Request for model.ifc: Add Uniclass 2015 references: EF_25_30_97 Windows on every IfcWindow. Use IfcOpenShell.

First a look at what the model holds.

```python
import ifcopenshell

model = ifcopenshell.open("model.ifc")
print(model.schema)
print("classifications:", [c.Name for c in model.by_type("IfcClassification")])
for ifc_class in ("IfcDoor", "IfcRoof", "IfcStair", "IfcWall", "IfcWindow"):
    print(ifc_class, len(model.by_type(ifc_class)))
```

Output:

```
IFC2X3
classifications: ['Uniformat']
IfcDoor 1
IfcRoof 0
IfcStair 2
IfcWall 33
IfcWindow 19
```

```python
import ifcopenshell
import ifcopenshell.api.classification

model = ifcopenshell.open("model.ifc")

# IFC2X3 requires Source and Edition and has no link from the project to the system.
system = model.create_entity("IfcClassification", Source="NBS", Edition="2015", Name="Uniclass 2015")

codes = {
    "IfcWindow": ("EF_25_30_97", "Windows"),
}
for ifc_class, (code, name) in codes.items():
    products = model.by_type(ifc_class)
    ifcopenshell.api.classification.add_reference(
        model, products=products, classification=system, identification=code, name=name
    )
    print(code, len(products))

model.write("model-out.ifc")
```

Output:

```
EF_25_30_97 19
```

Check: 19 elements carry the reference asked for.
